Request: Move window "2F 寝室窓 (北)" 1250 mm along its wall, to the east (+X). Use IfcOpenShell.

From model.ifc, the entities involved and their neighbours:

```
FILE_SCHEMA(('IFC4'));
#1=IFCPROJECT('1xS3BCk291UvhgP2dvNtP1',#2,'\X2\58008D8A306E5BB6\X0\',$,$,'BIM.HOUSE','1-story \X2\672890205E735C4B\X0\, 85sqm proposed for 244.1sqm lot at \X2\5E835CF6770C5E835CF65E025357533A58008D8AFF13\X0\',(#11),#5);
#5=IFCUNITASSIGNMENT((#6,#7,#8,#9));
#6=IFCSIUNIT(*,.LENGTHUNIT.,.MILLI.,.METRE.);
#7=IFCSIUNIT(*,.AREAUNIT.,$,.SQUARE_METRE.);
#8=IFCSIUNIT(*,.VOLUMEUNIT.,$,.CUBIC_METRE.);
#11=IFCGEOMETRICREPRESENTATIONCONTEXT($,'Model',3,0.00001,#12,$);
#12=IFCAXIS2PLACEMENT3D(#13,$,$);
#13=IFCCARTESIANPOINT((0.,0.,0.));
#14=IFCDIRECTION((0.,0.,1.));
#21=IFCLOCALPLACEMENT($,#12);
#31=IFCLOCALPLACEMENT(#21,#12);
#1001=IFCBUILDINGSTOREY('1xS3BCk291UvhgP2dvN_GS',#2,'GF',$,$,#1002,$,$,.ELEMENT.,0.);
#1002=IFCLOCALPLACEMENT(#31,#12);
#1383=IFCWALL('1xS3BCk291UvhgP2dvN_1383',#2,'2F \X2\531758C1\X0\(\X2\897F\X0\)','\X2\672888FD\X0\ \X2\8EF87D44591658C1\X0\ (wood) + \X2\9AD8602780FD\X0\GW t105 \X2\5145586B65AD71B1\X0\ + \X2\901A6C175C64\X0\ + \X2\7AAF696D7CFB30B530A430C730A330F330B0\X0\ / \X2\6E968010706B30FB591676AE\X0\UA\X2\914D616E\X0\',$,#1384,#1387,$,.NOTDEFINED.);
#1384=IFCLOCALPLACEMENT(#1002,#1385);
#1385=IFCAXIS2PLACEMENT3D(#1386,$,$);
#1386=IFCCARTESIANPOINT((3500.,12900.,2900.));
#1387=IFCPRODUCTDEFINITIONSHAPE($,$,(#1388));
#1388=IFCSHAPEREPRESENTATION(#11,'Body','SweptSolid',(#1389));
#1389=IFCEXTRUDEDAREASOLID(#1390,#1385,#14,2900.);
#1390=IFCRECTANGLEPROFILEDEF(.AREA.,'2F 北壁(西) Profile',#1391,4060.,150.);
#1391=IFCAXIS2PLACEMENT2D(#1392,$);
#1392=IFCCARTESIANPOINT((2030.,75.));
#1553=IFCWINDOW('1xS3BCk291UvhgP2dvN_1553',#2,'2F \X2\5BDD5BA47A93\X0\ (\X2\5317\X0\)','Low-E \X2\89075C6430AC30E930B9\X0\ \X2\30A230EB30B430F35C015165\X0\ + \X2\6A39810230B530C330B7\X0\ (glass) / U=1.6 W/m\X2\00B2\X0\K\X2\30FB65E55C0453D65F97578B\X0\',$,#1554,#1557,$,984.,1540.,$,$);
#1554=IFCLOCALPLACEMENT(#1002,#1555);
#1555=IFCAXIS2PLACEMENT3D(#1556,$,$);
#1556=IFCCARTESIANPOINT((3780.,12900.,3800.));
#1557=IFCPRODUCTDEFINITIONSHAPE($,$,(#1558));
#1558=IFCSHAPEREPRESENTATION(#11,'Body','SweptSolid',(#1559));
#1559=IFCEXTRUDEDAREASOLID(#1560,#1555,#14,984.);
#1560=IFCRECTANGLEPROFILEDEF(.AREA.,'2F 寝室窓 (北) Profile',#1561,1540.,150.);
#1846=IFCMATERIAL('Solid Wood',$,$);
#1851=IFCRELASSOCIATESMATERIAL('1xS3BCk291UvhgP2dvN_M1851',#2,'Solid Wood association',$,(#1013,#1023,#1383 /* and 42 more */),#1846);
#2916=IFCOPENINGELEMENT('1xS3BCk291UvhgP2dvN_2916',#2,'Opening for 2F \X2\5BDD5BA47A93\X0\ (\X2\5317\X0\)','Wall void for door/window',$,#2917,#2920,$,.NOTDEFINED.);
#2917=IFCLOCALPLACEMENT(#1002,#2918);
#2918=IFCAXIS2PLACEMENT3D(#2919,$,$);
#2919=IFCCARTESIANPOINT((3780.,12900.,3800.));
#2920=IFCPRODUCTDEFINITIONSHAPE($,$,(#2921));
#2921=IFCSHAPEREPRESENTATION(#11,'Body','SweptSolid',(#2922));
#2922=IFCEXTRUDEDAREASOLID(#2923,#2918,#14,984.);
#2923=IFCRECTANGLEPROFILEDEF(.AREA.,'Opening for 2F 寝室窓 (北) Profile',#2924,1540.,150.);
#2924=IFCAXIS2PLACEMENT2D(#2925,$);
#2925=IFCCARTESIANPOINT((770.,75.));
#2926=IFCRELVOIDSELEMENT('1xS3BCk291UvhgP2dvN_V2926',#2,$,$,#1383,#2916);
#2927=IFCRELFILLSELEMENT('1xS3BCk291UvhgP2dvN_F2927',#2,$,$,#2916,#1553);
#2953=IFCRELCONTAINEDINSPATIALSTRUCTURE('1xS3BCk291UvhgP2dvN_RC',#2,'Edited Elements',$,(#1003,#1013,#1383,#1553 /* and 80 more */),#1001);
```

```python
import ifcopenshell
import ifcopenshell.api.geometry
import ifcopenshell.util.placement

model = ifcopenshell.open("model.ifc")

window = model.by_id(1553)
opening = window.FillsVoids[0].RelatingOpeningElement
wall = opening.VoidsElements[0].RelatingBuildingElement

wall_matrix = ifcopenshell.util.placement.get_local_placement(wall.ObjectPlacement)
shift = wall_matrix[:3, 0] * 1250.0
before = ifcopenshell.util.placement.get_local_placement(window.ObjectPlacement)[:3, 3].copy()

# The window is not placed relative to its opening, so move both.
for product in (opening, window):
    matrix = ifcopenshell.util.placement.get_local_placement(product.ObjectPlacement)
    matrix[:3, 3] += shift
    ifcopenshell.api.geometry.edit_object_placement(model, product=product, matrix=matrix, is_si=False)

after = ifcopenshell.util.placement.get_local_placement(window.ObjectPlacement)[:3, 3]
print("window moved by", (after - before).round(3) + 0.0)

model.write("model-out.ifc")
```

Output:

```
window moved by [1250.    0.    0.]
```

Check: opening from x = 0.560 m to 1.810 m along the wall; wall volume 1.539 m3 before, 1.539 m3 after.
